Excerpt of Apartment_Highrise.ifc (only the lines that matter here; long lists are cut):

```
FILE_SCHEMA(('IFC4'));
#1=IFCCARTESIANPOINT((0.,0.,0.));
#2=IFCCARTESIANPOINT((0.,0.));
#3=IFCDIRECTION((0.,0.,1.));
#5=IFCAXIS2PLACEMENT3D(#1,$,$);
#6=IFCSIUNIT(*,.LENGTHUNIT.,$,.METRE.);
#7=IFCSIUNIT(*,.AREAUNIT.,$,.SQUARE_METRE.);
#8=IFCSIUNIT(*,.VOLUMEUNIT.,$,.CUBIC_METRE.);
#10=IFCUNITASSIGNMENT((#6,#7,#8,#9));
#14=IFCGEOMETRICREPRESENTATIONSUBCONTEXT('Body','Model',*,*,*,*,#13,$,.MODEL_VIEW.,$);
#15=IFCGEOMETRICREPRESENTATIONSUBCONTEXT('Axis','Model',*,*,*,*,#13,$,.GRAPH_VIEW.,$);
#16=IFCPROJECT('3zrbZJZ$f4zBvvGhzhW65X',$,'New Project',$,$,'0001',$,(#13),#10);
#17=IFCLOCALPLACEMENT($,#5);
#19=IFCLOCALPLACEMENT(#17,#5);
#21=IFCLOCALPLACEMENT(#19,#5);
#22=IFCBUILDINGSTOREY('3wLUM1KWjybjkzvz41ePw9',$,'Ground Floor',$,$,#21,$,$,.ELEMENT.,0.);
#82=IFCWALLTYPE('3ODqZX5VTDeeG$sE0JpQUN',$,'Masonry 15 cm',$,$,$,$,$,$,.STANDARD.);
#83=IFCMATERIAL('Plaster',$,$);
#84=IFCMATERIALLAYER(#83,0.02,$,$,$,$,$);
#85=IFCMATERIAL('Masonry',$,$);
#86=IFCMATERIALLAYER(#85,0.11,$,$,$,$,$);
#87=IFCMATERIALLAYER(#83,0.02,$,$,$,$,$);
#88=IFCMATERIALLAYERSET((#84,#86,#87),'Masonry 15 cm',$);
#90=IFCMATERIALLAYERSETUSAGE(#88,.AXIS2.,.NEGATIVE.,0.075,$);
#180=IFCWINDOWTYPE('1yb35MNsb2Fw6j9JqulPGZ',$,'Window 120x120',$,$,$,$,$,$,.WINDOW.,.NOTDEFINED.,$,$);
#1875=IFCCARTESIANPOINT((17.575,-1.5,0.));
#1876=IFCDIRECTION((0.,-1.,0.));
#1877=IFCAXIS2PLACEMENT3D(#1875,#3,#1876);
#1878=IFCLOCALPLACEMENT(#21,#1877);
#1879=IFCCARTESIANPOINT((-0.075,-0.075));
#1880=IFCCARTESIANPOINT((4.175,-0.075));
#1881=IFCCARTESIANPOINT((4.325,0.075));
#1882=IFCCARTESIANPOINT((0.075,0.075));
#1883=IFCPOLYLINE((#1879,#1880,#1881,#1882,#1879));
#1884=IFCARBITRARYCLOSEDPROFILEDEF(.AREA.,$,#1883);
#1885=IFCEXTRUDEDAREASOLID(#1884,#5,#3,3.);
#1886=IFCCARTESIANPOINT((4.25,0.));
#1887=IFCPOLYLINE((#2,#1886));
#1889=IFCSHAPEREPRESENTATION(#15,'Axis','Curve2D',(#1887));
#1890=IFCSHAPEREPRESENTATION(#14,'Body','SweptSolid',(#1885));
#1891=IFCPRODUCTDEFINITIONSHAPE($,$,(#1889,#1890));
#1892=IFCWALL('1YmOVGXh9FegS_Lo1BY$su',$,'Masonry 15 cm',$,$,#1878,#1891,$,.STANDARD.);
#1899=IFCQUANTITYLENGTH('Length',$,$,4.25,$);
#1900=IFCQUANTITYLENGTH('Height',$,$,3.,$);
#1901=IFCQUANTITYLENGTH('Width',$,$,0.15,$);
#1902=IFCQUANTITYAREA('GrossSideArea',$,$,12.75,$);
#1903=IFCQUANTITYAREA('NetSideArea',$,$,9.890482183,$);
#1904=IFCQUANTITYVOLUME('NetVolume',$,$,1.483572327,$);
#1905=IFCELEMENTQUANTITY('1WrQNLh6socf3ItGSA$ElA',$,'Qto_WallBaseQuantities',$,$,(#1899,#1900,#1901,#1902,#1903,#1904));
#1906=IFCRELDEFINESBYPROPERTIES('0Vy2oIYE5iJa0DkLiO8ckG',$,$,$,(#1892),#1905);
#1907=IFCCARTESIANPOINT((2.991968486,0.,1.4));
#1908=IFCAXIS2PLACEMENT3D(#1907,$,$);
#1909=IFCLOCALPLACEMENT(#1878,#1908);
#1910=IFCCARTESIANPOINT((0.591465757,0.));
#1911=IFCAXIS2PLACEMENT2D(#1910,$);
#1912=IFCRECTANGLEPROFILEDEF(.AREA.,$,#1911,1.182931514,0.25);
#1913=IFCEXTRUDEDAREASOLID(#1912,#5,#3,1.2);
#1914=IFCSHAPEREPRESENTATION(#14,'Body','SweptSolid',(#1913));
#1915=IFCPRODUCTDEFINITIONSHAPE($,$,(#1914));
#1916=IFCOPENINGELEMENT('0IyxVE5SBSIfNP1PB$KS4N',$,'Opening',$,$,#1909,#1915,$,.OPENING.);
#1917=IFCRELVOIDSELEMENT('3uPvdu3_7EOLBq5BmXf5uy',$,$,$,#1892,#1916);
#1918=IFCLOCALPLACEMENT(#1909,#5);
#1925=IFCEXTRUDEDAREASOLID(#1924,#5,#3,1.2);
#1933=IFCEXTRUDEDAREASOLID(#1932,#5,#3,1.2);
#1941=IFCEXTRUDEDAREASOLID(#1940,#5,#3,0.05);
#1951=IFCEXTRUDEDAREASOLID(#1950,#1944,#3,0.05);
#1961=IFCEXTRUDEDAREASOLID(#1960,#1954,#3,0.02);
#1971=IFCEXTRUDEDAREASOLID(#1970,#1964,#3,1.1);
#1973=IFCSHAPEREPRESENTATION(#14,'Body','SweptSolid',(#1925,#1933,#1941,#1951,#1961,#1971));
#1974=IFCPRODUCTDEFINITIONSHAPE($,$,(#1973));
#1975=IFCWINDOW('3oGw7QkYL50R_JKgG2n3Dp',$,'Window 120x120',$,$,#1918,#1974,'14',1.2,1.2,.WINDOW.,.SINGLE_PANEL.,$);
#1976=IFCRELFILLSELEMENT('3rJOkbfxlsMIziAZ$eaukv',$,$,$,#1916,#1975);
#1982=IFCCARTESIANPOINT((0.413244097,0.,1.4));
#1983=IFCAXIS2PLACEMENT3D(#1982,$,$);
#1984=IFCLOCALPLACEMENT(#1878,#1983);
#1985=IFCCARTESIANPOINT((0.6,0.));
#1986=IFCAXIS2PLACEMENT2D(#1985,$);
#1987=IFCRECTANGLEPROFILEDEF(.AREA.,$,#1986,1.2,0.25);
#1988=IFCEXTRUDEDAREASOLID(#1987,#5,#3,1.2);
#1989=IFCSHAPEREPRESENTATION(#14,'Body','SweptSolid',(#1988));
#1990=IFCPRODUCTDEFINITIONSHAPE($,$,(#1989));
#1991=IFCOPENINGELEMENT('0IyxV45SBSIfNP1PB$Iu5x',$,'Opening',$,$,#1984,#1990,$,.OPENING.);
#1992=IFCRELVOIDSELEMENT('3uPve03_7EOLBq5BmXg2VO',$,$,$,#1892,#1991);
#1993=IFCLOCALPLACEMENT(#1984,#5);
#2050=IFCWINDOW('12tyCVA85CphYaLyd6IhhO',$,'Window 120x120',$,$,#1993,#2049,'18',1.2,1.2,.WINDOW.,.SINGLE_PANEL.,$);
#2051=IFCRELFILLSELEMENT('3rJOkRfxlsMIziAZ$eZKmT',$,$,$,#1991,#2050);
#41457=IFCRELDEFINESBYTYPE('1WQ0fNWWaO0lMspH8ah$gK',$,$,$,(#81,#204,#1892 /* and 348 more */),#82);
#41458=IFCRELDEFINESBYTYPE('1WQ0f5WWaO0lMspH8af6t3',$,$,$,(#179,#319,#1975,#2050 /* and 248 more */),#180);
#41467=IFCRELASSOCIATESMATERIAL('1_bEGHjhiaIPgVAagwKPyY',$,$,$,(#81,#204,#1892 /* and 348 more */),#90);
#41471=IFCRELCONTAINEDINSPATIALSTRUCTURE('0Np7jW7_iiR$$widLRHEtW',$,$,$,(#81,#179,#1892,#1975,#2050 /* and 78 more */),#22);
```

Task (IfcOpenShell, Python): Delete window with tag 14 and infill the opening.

```python
import ifcopenshell
import ifcopenshell.api.feature
import ifcopenshell.api.pset
import ifcopenshell.api.root
import ifcopenshell.geom
import ifcopenshell.util.element
import ifcopenshell.util.shape
import ifcopenshell.util.unit

model = ifcopenshell.open("Apartment_Highrise.ifc")
area_scale = ifcopenshell.util.unit.calculate_unit_scale(model, "AREAUNIT")
volume_scale = ifcopenshell.util.unit.calculate_unit_scale(model, "VOLUMEUNIT")
settings = ifcopenshell.geom.settings()


def volume(element):
    """Net volume in cubic metres, openings subtracted."""
    shape = ifcopenshell.geom.create_shape(settings, element)
    return ifcopenshell.util.shape.get_volume(shape.geometry)


window = model.by_guid("3oGw7QkYL50R_JKgG2n3Dp")
opening = window.FillsVoids[0].RelatingOpeningElement
wall = opening.VoidsElements[0].RelatingBuildingElement
before = volume(wall)

ifcopenshell.api.root.remove_product(model, product=window)
ifcopenshell.api.feature.remove_feature(model, feature=opening)

after = volume(wall)
thickness = 0.15  # wall thickness in metres

# Update the wall's stored quantities.
qto = model.by_id(ifcopenshell.util.element.get_pset(wall, "Qto_WallBaseQuantities", should_inherit=False)["id"])
ifcopenshell.api.pset.edit_qto(model, qto=qto, properties={
    "NetSideArea": after / thickness / area_scale,
    "NetVolume": after / volume_scale,
})

print(f"wall volume {before:.3f} -> {after:.3f} m3")

model.write("Apartment_Highrise_edited.ifc")
```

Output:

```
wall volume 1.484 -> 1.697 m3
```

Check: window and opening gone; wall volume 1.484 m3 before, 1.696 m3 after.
